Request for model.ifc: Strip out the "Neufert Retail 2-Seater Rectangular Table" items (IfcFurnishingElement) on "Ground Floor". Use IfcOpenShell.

First a look at what the model holds.

```python
import ifcopenshell
import ifcopenshell.util.element

model = ifcopenshell.open("model.ifc")
print(model.schema)
storey = next(s for s in model.by_type("IfcBuildingStorey") if s.Name == "Ground Floor")
furniture = [e for e in ifcopenshell.util.element.get_decomposition(storey) if e.is_a("IfcFurnishingElement")]
seen = {}
for e in furniture:
    element_type = ifcopenshell.util.element.get_type(e)
    name = element_type.Name if element_type not in (None, e) else None
    seen[name] = seen.get(name, 0) + 1
for name, count in sorted(seen.items(), key=str):
    print(count, "x", name)
```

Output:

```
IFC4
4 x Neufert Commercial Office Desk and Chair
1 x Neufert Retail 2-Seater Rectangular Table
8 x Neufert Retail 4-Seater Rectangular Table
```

```python
import ifcopenshell
import ifcopenshell.api.root
import ifcopenshell.util.element

model = ifcopenshell.open("model.ifc")

storey = next(s for s in model.by_type("IfcBuildingStorey") if s.Name == "Ground Floor")
furniture = [e for e in ifcopenshell.util.element.get_decomposition(storey) if e.is_a("IfcFurnishingElement")]
targets = [e for e in furniture if (t := ifcopenshell.util.element.get_type(e)) not in (None, e) and t.Name == "Neufert Retail 2-Seater Rectangular Table"]

for e in targets:
    ifcopenshell.api.root.remove_product(model, product=e)
print(len(targets), "removed")

model.write("model_v2.ifc")
```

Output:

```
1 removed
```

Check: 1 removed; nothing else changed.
